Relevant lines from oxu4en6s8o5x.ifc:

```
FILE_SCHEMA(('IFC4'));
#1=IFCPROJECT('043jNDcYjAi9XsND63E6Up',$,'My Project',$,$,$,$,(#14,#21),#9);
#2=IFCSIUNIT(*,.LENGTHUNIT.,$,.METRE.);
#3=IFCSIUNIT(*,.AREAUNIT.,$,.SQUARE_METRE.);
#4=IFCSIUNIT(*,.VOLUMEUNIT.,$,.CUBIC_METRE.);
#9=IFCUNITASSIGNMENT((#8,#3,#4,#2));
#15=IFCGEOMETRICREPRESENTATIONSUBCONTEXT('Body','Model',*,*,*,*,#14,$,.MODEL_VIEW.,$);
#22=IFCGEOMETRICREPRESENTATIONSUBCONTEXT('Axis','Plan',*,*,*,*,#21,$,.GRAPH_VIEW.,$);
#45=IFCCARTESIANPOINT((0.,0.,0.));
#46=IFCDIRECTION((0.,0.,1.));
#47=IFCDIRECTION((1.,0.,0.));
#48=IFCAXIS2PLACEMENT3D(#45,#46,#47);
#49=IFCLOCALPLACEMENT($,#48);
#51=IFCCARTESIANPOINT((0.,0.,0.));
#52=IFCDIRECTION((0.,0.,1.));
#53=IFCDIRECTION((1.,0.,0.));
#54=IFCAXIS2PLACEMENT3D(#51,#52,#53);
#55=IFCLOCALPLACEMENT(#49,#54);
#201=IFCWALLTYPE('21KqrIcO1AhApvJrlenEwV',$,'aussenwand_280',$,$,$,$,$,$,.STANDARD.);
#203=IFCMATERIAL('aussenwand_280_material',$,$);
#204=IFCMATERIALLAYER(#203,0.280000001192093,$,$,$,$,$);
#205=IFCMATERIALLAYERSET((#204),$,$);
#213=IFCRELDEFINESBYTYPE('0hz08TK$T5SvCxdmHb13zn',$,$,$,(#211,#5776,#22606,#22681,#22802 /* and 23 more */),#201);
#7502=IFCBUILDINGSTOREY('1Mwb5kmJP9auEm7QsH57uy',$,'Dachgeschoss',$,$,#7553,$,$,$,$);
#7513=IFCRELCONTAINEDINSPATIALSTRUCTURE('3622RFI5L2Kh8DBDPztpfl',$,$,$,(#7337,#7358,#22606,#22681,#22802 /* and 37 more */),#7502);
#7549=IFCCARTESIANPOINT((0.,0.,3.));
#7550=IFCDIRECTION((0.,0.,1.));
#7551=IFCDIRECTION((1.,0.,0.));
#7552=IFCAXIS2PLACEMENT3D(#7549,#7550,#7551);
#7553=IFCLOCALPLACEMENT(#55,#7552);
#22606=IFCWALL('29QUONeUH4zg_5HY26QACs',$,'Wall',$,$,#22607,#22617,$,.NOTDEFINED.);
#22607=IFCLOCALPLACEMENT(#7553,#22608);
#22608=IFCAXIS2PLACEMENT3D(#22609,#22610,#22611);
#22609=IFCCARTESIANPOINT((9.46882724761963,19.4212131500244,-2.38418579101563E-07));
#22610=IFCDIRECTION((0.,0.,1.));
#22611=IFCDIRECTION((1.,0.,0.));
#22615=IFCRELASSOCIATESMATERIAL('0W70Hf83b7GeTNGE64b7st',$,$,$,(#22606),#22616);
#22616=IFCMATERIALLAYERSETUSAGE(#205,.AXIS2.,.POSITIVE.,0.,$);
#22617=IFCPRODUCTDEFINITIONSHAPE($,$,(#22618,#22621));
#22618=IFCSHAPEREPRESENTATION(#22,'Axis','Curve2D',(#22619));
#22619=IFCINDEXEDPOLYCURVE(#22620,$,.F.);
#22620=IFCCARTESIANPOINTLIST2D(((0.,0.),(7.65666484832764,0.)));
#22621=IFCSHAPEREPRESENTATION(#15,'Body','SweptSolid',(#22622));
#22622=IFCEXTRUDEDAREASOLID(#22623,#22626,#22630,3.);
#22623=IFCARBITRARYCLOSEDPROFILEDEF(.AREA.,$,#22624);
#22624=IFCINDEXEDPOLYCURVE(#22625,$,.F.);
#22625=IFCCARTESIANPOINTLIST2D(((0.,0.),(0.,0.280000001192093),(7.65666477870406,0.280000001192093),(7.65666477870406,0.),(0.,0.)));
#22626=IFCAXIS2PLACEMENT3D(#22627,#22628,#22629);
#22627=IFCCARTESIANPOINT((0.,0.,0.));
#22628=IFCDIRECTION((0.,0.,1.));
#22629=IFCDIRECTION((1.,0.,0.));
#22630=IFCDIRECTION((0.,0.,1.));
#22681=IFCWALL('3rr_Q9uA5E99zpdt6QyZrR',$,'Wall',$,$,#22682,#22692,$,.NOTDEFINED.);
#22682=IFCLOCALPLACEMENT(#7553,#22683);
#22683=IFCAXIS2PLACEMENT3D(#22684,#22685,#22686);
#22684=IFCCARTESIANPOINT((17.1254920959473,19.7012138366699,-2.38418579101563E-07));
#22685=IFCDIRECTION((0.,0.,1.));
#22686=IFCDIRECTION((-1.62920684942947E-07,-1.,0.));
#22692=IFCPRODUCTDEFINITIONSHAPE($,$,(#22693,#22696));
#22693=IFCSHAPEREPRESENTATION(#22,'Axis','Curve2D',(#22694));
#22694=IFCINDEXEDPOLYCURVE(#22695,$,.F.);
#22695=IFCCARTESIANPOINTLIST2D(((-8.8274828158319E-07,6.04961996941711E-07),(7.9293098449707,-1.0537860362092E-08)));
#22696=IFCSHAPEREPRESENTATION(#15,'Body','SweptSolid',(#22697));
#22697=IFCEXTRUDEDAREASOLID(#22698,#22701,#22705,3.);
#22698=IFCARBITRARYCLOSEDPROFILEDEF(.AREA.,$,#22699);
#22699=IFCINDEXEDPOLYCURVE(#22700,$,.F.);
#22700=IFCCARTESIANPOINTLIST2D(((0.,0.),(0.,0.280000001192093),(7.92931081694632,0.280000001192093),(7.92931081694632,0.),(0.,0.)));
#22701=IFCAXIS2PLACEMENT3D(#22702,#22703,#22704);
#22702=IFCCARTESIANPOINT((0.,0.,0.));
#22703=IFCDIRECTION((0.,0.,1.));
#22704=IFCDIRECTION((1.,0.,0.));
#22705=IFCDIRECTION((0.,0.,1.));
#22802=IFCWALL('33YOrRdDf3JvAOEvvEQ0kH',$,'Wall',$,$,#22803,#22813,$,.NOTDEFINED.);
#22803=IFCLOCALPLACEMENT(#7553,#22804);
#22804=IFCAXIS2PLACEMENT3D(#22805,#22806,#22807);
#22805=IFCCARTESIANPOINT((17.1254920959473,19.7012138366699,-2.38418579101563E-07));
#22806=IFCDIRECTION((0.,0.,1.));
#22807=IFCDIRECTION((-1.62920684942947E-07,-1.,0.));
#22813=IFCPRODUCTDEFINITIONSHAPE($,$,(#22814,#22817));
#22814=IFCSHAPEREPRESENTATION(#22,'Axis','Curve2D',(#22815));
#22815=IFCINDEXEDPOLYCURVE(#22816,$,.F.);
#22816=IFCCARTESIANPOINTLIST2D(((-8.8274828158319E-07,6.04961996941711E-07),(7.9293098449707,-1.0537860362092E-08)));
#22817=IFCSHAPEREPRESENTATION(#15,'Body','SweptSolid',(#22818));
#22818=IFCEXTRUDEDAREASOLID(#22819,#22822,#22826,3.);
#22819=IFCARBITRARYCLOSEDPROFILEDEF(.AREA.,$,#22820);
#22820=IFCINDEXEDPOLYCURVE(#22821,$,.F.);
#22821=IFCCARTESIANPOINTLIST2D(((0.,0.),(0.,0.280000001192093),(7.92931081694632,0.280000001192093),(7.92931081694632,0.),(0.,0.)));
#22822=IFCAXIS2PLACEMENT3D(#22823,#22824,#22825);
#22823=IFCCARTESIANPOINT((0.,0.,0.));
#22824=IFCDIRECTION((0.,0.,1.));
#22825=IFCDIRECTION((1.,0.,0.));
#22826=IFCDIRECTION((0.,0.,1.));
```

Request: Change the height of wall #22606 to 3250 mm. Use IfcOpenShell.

```python
import ifcopenshell
import ifcopenshell.geom
import ifcopenshell.util.representation
import ifcopenshell.util.shape
import ifcopenshell.util.unit

model = ifcopenshell.open("oxu4en6s8o5x.ifc")
unit_scale = ifcopenshell.util.unit.calculate_unit_scale(model)
settings = ifcopenshell.geom.settings()


def volume(element):
    """Net volume in cubic metres, openings subtracted."""
    shape = ifcopenshell.geom.create_shape(settings, element)
    return ifcopenshell.util.shape.get_volume(shape.geometry)


wall = model.by_id(22606)
before = volume(wall)

body = ifcopenshell.util.representation.get_representation(wall, "Model", "Body")
solid = body.Items[0]
old_height = solid.Depth
solid.Depth = 3.25 / unit_scale
after = volume(wall)

print(f"height {old_height:g} -> {solid.Depth:g}, volume {before:.3f} -> {after:.3f} m3")

model.write("oxu4en6s8o5x_edited.ifc")
```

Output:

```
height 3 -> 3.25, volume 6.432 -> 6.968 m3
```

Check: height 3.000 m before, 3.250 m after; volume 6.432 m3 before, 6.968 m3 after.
